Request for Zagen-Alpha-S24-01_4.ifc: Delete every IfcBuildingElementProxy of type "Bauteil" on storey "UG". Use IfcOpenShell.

First a look at what the model holds.

```python
import ifcopenshell
import ifcopenshell.util.element

model = ifcopenshell.open("Zagen-Alpha-S24-01_4.ifc")
print(model.schema)
storey = next(s for s in model.by_type("IfcBuildingStorey") if s.Name == "UG")
proxies = [e for e in ifcopenshell.util.element.get_decomposition(storey) if e.is_a("IfcBuildingElementProxy")]
seen = {}
for e in proxies:
    element_type = ifcopenshell.util.element.get_type(e)
    name = element_type.Name if element_type not in (None, e) else None
    seen[name] = seen.get(name, 0) + 1
for name, count in sorted(seen.items(), key=str):
    print(count, "x", name)
```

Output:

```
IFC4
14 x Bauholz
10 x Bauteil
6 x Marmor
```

```python
import ifcopenshell
import ifcopenshell.api.root
import ifcopenshell.util.element

model = ifcopenshell.open("Zagen-Alpha-S24-01_4.ifc")

storey = next(s for s in model.by_type("IfcBuildingStorey") if s.Name == "UG")
proxies = [e for e in ifcopenshell.util.element.get_decomposition(storey) if e.is_a("IfcBuildingElementProxy")]
targets = [e for e in proxies if (t := ifcopenshell.util.element.get_type(e)) not in (None, e) and t.Name == "Bauteil"]

for e in targets:
    ifcopenshell.api.root.remove_product(model, product=e)
print(len(targets), "removed")

model.write("Zagen-Alpha-S24-01_4_v2.ifc")
```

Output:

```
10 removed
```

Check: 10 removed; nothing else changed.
